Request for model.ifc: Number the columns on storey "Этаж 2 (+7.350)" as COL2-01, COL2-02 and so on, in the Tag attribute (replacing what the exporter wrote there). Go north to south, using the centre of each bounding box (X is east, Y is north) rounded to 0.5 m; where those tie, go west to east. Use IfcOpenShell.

First a look at what the model holds.

```python
import ifcopenshell
import ifcopenshell.util.element
import ifcopenshell.util.placement

model = ifcopenshell.open("model.ifc")
print(model.schema)
storey = next(s for s in model.by_type("IfcBuildingStorey") if s.Name == "Этаж 2 (+7.350)")
columns = [e for e in ifcopenshell.util.element.get_decomposition(storey) if e.is_a("IfcColumn")]
for e in sorted(columns, key=lambda e: e.id()):
    origin = ifcopenshell.util.placement.get_local_placement(e.ObjectPlacement)[:3, 3]
    print(e.id(), e.Tag, e.Name, origin.round(2) + 0.0, sep=" | ")
```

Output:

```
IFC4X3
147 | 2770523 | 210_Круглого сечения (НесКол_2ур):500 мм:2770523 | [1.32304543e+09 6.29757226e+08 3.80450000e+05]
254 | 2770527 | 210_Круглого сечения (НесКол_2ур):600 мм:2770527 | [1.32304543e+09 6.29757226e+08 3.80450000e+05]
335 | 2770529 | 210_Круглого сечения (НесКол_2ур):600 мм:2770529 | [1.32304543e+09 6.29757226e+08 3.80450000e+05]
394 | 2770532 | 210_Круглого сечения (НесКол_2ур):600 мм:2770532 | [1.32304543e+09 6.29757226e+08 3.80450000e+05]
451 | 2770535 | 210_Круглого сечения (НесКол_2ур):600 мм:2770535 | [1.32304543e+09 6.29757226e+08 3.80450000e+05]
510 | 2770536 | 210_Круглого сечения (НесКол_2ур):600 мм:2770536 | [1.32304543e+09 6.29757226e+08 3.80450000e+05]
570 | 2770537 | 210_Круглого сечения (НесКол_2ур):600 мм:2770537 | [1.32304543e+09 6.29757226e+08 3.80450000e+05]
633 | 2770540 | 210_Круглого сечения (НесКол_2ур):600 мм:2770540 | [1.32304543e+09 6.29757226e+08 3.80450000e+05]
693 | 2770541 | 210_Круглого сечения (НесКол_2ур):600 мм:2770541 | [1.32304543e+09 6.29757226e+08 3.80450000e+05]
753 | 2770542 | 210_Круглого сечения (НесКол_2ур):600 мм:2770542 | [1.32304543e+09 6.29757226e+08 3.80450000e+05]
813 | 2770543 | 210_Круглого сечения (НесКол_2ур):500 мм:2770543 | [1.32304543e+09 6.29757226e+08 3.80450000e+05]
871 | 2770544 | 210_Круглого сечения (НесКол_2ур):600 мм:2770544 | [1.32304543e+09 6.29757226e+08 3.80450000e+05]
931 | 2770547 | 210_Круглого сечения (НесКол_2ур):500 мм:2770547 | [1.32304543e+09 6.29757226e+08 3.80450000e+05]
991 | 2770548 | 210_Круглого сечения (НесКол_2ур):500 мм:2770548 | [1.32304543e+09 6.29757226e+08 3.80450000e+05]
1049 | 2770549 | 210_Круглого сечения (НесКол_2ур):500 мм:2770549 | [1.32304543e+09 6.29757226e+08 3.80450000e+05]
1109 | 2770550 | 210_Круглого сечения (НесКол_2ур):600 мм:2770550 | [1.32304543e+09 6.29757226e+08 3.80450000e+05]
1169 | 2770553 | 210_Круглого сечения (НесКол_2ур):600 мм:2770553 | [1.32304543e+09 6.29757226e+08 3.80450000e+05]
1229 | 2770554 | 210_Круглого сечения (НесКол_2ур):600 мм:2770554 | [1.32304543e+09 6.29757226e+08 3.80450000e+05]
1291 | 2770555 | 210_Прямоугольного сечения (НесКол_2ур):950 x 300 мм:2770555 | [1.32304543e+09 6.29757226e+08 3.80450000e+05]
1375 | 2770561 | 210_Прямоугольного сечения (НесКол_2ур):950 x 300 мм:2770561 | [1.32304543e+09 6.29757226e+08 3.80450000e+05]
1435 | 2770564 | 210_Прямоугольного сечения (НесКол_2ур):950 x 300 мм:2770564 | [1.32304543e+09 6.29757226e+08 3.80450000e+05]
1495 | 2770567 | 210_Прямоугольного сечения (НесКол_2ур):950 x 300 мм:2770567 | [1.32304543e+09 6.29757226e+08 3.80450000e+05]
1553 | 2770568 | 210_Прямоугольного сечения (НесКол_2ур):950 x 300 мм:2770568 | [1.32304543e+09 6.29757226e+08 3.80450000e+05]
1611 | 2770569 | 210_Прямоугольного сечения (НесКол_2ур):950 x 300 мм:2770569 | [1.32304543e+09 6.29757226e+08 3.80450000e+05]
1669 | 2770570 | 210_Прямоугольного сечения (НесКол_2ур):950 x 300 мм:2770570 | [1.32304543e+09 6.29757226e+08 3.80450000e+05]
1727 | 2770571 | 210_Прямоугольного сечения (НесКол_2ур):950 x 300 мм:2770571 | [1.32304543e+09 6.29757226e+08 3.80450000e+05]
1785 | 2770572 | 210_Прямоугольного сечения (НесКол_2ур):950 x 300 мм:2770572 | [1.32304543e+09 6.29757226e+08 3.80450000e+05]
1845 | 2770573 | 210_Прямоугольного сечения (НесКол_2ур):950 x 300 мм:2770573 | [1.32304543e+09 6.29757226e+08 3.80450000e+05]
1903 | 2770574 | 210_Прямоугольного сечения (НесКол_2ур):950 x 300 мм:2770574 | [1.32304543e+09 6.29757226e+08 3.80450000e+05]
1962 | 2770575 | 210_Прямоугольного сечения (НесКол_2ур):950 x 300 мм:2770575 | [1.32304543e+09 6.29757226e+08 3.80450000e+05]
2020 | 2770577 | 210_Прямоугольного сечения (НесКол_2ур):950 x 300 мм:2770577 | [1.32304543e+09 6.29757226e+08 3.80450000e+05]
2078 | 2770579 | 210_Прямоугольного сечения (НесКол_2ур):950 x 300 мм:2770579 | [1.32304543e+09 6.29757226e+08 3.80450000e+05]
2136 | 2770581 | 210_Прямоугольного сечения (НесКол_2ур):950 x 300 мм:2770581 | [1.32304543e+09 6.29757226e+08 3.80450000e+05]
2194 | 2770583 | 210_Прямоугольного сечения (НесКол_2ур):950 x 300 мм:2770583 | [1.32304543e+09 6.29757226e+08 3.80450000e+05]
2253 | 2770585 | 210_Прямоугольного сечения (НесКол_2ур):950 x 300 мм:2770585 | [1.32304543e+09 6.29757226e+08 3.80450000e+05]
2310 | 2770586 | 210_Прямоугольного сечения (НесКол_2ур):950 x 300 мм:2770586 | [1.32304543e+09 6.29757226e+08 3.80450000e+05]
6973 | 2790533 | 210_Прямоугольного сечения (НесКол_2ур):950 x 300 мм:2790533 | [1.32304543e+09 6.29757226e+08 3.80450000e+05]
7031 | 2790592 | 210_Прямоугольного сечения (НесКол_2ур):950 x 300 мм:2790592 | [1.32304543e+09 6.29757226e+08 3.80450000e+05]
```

```python
import ifcopenshell
import ifcopenshell.geom
import ifcopenshell.util.element
import ifcopenshell.util.shape

model = ifcopenshell.open("model.ifc")
settings = ifcopenshell.geom.settings()
settings.set("use-world-coords", True)


def centre(element):
    shape = ifcopenshell.geom.create_shape(settings, element)
    return ifcopenshell.util.shape.get_bbox_centroid(shape.geometry)


storey = next(s for s in model.by_type("IfcBuildingStorey") if s.Name == "Этаж 2 (+7.350)")
columns = [e for e in ifcopenshell.util.element.get_decomposition(storey) if e.is_a("IfcColumn")]

# Insertion points can sit at a corner or the storey origin, so sort by the geometry (in metres).
centres = {e: centre(e) for e in columns}
columns.sort(key=lambda e: (-round(centres[e][1] / 0.5), centres[e][0]))

for i, e in enumerate(columns, start=1):
    number = f"COL2-{i:02d}"
    e.Tag = number
    print(e.id(), number)

model.write("model_edited.ifc")
```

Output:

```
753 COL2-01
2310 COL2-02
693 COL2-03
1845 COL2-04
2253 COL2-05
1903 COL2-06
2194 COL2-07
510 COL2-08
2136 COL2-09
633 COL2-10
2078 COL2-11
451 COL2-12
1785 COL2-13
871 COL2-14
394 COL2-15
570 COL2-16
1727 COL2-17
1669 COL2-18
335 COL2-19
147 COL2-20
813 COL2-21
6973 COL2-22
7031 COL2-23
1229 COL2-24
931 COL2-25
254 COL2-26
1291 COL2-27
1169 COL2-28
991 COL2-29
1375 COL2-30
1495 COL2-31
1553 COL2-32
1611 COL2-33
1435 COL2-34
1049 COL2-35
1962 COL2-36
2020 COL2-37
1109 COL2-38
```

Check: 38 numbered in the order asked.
